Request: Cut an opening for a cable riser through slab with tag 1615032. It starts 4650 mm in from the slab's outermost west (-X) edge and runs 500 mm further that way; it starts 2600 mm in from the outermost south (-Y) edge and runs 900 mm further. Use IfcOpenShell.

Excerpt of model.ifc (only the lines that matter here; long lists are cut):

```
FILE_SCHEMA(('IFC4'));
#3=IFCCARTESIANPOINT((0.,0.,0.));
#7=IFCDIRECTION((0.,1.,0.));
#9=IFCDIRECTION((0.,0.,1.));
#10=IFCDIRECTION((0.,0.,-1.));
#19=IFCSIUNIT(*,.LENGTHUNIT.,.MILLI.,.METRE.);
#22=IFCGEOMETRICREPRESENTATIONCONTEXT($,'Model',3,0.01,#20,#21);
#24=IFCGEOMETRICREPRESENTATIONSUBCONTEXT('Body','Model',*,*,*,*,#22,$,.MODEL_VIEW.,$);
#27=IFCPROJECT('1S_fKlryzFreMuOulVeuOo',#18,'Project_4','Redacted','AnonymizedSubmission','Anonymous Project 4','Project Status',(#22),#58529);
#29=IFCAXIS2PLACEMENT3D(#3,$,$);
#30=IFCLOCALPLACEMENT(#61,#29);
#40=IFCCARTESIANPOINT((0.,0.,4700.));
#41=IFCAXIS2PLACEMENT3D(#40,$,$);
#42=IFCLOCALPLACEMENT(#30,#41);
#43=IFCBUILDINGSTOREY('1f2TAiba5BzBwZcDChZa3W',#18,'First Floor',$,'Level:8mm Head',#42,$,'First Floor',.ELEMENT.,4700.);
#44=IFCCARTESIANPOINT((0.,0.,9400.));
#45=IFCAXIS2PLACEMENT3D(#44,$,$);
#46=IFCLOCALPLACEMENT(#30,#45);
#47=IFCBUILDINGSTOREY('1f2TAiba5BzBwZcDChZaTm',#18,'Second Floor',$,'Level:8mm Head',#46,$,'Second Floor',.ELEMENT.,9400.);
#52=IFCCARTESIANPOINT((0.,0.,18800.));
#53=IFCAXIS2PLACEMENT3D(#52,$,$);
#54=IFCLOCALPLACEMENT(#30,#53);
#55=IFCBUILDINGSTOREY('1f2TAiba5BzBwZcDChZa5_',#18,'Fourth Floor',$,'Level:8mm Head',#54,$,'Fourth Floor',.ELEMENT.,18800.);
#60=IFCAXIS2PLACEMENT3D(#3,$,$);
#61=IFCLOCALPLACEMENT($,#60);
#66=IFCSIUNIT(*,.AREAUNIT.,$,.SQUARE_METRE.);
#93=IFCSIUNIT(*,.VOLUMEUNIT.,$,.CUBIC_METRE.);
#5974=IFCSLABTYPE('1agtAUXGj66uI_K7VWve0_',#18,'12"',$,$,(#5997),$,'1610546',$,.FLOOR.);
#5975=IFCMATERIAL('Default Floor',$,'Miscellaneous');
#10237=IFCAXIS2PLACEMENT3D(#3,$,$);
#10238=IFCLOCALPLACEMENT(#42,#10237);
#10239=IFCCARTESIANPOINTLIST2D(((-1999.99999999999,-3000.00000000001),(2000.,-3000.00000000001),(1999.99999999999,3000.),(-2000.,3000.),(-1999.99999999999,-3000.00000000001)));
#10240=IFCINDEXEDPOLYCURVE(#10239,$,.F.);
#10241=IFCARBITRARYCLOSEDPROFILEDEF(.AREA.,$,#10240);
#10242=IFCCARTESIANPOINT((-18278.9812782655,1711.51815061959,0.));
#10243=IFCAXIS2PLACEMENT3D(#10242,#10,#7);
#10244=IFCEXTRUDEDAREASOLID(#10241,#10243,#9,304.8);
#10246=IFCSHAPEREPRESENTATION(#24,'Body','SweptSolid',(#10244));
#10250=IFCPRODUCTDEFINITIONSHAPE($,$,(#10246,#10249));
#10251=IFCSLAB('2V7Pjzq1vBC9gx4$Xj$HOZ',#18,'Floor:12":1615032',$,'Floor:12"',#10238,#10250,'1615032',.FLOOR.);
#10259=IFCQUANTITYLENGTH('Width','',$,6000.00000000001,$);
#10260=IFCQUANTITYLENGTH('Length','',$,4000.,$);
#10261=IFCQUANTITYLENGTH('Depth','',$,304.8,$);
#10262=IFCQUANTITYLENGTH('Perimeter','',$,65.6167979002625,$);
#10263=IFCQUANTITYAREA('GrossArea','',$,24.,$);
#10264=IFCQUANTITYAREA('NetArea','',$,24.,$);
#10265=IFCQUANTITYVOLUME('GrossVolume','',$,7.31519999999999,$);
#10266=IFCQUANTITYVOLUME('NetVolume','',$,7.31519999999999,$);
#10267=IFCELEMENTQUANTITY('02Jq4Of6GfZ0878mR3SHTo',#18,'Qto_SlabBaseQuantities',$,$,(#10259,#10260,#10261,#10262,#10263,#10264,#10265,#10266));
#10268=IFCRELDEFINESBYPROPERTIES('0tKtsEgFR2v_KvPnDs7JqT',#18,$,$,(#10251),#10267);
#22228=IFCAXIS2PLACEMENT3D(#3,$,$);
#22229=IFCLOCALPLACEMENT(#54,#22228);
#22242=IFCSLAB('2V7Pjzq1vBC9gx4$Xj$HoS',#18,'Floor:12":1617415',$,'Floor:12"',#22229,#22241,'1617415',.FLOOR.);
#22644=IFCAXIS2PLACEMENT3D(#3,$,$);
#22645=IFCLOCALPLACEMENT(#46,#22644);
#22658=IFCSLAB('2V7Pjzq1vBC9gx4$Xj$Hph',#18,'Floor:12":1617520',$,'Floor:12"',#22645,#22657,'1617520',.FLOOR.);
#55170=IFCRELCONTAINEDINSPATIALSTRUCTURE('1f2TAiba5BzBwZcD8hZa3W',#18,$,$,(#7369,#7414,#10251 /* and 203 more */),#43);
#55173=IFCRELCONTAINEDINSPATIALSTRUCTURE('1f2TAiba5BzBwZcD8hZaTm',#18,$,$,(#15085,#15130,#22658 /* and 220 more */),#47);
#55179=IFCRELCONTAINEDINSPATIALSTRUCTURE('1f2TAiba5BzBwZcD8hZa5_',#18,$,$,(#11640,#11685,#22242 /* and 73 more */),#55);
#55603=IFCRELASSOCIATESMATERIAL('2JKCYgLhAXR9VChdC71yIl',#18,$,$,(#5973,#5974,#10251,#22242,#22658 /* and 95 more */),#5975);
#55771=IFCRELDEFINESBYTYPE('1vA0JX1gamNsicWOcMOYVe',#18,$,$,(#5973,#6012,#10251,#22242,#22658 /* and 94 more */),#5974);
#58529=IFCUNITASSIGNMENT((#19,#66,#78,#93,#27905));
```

```python
import numpy as np
import ifcopenshell
import ifcopenshell.api.feature
import ifcopenshell.api.geometry
import ifcopenshell.api.pset
import ifcopenshell.api.root
import ifcopenshell.geom
import ifcopenshell.util.element
import ifcopenshell.util.placement
import ifcopenshell.util.representation
import ifcopenshell.util.shape
import ifcopenshell.util.unit

model = ifcopenshell.open("model.ifc")
unit_scale = ifcopenshell.util.unit.calculate_unit_scale(model)
area_scale = ifcopenshell.util.unit.calculate_unit_scale(model, "AREAUNIT")
volume_scale = ifcopenshell.util.unit.calculate_unit_scale(model, "VOLUMEUNIT")
settings = ifcopenshell.geom.settings()


def volume(element):
    """Net volume in cubic metres, openings subtracted."""
    shape = ifcopenshell.geom.create_shape(settings, element)
    return ifcopenshell.util.shape.get_volume(shape.geometry)


slab = model.by_guid("2V7Pjzq1vBC9gx4$Xj$HOZ")
before = volume(slab)

# Extent in the slab's own axes, in metres. The edges named are its -X and -Y sides.
slab_shape = ifcopenshell.geom.create_shape(settings, slab)
vertices = ifcopenshell.util.shape.get_vertices(slab_shape.geometry)
x_min, y_min, bottom = vertices.min(axis=0)
top = vertices[:, 2].max()

opening = ifcopenshell.api.root.create_entity(model, ifc_class="IfcOpeningElement", name="Cable riser opening", predefined_type="OPENING")
context = ifcopenshell.util.representation.get_context(model, "Model", "Body", "MODEL_VIEW")
width, depth = 0.5, 0.9
outline = [(0.0, 0.0), (width, 0.0), (width, depth), (0.0, depth), (0.0, 0.0)]
# Overshoot both faces by 50 mm so the cut is clean.
shape = ifcopenshell.api.geometry.add_slab_representation(
    model, context=context, depth=top - bottom + 0.1, polyline=outline
)
ifcopenshell.api.geometry.assign_representation(model, product=opening, representation=shape)

matrix = ifcopenshell.util.placement.get_local_placement(slab.ObjectPlacement)
matrix[:, 3] = matrix @ np.append(np.array([x_min + 4.65, y_min + 2.6, bottom - 0.05]) / unit_scale, 1.0)
ifcopenshell.api.geometry.edit_object_placement(model, product=opening, matrix=matrix, is_si=False)
ifcopenshell.api.feature.add_feature(model, feature=opening, element=slab)

after = volume(slab)

# Update the slab's stored quantities.
qto = model.by_id(ifcopenshell.util.element.get_pset(slab, "Qto_SlabBaseQuantities", should_inherit=False)["id"])
ifcopenshell.api.pset.edit_qto(model, qto=qto, properties={
    "NetArea": after / (top - bottom) / area_scale,
    "NetVolume": after / volume_scale,
})

print(f"slab volume {before:.3f} -> {after:.3f} m3")

model.write("model_updated.ifc")
```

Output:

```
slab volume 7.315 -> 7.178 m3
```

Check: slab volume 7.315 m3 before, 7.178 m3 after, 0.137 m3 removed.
